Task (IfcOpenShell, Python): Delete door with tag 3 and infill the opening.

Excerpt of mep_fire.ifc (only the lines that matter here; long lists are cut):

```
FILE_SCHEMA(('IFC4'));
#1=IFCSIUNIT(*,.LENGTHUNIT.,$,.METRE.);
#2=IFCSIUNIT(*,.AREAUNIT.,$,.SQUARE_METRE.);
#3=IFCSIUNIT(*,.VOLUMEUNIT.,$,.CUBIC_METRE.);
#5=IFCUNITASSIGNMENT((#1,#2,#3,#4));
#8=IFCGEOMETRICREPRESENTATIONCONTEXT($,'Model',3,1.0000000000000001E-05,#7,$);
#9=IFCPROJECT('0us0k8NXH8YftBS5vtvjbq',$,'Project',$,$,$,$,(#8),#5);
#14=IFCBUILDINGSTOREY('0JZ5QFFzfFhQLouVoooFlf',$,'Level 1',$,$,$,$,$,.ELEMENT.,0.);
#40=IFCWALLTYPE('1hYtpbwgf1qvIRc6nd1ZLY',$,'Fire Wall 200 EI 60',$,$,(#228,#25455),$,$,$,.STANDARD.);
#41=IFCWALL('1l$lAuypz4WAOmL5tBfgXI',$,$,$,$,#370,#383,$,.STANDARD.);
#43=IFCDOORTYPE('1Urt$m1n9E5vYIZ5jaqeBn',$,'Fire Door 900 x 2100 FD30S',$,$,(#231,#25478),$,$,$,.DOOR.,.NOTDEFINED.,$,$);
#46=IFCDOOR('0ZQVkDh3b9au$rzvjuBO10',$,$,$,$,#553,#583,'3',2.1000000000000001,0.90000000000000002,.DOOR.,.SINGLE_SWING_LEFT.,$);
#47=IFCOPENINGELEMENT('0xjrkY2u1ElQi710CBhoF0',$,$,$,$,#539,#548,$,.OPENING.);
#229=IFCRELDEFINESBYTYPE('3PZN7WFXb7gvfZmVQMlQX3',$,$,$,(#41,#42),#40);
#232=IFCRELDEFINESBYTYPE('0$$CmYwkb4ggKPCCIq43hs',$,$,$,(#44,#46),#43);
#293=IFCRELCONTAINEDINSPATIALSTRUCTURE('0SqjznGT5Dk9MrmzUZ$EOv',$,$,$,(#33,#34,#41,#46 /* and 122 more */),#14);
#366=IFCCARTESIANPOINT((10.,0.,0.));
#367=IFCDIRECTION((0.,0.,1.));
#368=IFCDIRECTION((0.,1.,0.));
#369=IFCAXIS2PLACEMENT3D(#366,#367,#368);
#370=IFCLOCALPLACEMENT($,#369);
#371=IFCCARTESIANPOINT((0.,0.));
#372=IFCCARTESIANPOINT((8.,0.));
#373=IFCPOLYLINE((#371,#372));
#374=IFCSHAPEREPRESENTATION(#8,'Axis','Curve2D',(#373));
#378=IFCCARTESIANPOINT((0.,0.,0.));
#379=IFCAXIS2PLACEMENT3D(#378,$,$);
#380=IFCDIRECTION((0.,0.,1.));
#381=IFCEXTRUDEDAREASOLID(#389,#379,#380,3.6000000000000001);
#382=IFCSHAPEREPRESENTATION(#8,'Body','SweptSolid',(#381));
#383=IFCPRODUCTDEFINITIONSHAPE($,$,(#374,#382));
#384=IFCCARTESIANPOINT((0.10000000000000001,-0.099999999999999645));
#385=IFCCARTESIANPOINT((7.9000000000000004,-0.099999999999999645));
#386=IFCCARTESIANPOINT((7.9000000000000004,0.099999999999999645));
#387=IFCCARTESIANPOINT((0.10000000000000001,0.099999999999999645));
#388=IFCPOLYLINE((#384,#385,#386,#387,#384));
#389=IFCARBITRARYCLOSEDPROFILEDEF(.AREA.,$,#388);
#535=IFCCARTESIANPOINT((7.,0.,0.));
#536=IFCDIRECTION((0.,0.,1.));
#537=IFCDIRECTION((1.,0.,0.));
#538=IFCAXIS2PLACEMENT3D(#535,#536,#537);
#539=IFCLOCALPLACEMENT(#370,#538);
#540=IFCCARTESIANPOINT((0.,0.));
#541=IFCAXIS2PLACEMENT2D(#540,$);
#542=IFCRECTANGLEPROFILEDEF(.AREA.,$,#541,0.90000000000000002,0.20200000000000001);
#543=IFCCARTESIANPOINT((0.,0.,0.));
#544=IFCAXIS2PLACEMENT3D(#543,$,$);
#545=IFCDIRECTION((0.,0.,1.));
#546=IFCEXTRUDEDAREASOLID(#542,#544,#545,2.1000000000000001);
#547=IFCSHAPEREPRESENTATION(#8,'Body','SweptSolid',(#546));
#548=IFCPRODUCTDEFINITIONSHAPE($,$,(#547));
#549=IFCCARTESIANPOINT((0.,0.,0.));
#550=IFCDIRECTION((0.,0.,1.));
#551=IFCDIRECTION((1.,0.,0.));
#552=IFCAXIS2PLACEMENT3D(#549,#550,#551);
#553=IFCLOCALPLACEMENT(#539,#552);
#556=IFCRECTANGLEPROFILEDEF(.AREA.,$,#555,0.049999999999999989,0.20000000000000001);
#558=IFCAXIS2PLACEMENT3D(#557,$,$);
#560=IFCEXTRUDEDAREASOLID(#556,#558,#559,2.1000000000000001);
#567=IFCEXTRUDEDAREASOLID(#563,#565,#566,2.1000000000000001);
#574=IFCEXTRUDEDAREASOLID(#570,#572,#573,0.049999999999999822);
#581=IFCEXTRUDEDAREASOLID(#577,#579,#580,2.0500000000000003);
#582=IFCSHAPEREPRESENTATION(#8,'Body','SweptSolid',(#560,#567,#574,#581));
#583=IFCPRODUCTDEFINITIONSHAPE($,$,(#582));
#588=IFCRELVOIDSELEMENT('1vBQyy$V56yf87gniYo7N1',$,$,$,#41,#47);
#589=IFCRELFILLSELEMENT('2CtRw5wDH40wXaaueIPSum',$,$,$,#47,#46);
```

```python
import ifcopenshell
import ifcopenshell.api.feature
import ifcopenshell.api.root
import ifcopenshell.geom
import ifcopenshell.util.shape

model = ifcopenshell.open("mep_fire.ifc")
settings = ifcopenshell.geom.settings()


def volume(element):
    """Net volume in cubic metres, openings subtracted."""
    shape = ifcopenshell.geom.create_shape(settings, element)
    return ifcopenshell.util.shape.get_volume(shape.geometry)


door = model.by_guid("0ZQVkDh3b9au$rzvjuBO10")
opening = door.FillsVoids[0].RelatingOpeningElement
wall = opening.VoidsElements[0].RelatingBuildingElement
before = volume(wall)

ifcopenshell.api.root.remove_product(model, product=door)
ifcopenshell.api.feature.remove_feature(model, feature=opening)

after = volume(wall)

print(f"wall volume {before:.3f} -> {after:.3f} m3")

model.write("mep_fire_rev.ifc")
```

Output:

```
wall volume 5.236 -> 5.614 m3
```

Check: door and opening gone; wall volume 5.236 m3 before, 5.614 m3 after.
